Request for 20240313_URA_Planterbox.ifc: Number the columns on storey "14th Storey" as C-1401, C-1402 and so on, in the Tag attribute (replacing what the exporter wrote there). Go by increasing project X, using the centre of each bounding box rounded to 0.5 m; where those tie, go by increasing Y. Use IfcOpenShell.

First a look at what the model holds.

```python
import ifcopenshell
import ifcopenshell.util.element
import ifcopenshell.util.placement

model = ifcopenshell.open("20240313_URA_Planterbox.ifc")
print(model.schema)
storey = next(s for s in model.by_type("IfcBuildingStorey") if s.Name == "14th Storey")
columns = [e for e in ifcopenshell.util.element.get_decomposition(storey) if e.is_a("IfcColumn")]
for e in sorted(columns, key=lambda e: e.id()):
    origin = ifcopenshell.util.placement.get_local_placement(e.ObjectPlacement)[:3, 3]
    print(e.id(), e.Tag, e.Name, origin.round(2) + 0.0, sep=" | ")
```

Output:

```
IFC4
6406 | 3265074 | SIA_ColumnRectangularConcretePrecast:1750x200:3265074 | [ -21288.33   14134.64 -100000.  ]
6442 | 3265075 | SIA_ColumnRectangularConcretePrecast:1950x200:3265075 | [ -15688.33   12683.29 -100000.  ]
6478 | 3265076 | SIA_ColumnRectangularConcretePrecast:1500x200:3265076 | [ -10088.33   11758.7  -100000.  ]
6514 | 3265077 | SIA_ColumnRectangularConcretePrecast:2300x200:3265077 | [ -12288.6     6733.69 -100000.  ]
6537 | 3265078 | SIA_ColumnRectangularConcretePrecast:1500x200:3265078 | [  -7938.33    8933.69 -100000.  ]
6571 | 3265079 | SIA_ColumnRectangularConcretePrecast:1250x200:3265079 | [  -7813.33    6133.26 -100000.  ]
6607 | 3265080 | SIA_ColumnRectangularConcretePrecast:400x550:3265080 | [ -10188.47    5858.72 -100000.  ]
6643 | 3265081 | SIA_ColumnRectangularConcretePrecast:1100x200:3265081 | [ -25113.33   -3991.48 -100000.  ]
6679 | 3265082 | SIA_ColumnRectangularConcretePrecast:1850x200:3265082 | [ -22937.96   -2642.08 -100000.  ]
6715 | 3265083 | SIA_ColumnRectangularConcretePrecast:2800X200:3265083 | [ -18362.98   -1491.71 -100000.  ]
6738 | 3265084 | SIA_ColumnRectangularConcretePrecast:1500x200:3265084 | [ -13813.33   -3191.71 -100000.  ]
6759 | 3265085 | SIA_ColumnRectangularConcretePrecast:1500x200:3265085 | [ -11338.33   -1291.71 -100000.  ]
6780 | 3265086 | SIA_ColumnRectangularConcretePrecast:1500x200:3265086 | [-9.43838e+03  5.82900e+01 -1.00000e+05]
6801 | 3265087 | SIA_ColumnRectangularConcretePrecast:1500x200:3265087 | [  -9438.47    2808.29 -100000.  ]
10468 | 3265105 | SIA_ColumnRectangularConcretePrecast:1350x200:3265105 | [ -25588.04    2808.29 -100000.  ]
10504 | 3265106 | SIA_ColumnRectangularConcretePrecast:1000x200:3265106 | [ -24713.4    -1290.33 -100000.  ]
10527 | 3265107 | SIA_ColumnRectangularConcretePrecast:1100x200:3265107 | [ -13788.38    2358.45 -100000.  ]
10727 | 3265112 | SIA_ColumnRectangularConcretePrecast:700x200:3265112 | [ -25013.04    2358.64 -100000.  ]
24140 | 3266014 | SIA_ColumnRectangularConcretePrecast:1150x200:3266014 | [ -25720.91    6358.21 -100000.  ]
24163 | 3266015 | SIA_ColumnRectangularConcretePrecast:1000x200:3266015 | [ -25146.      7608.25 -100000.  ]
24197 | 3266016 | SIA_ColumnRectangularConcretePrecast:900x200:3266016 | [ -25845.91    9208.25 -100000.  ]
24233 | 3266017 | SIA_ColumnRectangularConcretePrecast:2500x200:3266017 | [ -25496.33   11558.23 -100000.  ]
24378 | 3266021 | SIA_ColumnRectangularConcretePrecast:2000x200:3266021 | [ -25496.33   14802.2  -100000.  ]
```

```python
import ifcopenshell
import ifcopenshell.geom
import ifcopenshell.util.element
import ifcopenshell.util.shape

model = ifcopenshell.open("20240313_URA_Planterbox.ifc")
settings = ifcopenshell.geom.settings()
settings.set("use-world-coords", True)


def centre(element):
    shape = ifcopenshell.geom.create_shape(settings, element)
    return ifcopenshell.util.shape.get_bbox_centroid(shape.geometry)


storey = next(s for s in model.by_type("IfcBuildingStorey") if s.Name == "14th Storey")
columns = [e for e in ifcopenshell.util.element.get_decomposition(storey) if e.is_a("IfcColumn")]

# Insertion points can sit at a corner or the storey origin, so sort by the geometry (in metres).
centres = {e: centre(e) for e in columns}
columns.sort(key=lambda e: (round(centres[e][0] / 0.5), centres[e][1]))

for i, e in enumerate(columns, start=1):
    number = f"C-14{i:02d}"
    e.Tag = number
    print(e.id(), number)

model.write("20240313_URA_Planterbox_rev.ifc")
```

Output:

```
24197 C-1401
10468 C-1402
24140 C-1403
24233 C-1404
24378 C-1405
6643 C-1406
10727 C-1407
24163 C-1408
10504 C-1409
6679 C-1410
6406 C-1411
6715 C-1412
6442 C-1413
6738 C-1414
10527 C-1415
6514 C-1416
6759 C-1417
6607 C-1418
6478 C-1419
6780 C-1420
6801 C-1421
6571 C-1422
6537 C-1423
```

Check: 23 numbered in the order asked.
